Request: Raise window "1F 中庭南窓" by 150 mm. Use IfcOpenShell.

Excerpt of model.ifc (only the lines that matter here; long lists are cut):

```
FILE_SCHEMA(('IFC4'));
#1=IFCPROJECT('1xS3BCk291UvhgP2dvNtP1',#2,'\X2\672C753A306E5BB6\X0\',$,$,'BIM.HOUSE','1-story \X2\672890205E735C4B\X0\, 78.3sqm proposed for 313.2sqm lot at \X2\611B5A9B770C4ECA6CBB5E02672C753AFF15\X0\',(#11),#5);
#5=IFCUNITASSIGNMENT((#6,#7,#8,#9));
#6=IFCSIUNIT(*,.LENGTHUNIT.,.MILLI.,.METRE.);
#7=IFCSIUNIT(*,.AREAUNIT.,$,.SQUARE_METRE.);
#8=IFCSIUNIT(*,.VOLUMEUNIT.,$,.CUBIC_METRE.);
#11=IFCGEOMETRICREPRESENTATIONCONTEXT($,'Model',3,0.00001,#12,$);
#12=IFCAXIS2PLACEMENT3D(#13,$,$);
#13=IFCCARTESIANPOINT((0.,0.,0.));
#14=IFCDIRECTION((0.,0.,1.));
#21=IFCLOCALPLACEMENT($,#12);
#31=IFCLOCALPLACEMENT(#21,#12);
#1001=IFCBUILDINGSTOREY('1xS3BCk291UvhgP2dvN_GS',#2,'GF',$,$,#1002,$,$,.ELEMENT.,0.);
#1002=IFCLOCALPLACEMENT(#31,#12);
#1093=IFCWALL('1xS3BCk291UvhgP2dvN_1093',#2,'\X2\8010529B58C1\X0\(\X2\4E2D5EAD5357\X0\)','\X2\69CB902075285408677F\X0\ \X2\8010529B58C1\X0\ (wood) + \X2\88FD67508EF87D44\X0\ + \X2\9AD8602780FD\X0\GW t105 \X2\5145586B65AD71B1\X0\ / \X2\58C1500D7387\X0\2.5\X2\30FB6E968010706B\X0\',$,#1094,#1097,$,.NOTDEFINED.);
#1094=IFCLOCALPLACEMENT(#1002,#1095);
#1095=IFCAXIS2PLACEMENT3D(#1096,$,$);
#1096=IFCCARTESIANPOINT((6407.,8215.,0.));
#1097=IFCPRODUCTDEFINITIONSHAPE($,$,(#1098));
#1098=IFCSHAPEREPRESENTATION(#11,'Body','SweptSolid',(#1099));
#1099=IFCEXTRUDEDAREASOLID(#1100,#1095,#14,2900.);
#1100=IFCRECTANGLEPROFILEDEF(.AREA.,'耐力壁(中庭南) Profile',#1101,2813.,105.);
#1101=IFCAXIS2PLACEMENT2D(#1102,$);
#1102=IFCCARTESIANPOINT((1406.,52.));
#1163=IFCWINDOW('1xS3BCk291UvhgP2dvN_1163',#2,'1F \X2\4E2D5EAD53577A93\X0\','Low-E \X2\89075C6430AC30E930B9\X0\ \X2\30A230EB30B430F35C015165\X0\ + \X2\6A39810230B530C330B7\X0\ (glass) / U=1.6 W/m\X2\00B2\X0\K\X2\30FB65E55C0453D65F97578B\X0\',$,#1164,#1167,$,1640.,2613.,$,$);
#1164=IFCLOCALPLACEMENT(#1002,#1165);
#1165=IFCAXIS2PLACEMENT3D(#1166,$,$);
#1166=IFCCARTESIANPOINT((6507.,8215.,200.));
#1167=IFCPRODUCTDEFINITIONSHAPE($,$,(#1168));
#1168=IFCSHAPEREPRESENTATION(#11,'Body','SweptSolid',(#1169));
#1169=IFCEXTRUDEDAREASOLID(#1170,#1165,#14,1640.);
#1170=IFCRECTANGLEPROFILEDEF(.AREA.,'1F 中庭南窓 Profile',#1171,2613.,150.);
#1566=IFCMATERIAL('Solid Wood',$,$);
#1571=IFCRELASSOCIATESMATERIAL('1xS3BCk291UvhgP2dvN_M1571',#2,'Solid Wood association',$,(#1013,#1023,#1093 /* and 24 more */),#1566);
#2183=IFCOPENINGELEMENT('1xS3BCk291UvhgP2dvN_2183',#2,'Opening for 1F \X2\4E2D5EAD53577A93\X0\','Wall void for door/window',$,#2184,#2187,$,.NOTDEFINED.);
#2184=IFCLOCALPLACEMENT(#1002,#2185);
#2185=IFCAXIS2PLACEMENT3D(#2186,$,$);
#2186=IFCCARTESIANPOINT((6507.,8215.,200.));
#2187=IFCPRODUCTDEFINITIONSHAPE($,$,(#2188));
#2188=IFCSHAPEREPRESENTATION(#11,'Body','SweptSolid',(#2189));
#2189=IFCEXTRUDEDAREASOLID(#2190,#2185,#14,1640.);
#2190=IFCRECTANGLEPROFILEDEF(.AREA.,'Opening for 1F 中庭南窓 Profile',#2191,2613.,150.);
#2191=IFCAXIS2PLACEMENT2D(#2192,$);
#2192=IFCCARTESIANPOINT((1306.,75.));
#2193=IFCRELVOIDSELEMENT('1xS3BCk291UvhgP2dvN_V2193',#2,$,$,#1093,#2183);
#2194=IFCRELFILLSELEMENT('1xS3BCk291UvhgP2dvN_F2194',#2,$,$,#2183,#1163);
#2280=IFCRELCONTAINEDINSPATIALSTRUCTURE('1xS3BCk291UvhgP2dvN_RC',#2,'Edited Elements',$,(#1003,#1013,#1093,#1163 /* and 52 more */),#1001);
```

```python
import numpy as np
import ifcopenshell
import ifcopenshell.api.geometry
import ifcopenshell.util.placement
import ifcopenshell.util.unit

model = ifcopenshell.open("model.ifc")
unit_scale = ifcopenshell.util.unit.calculate_unit_scale(model)

window = model.by_guid("1xS3BCk291UvhgP2dvN_1163")
opening = window.FillsVoids[0].RelatingOpeningElement
dz = 0.15 / unit_scale

shift = np.array([0.0, 0.0, dz])
# The window is not placed relative to its opening, so move both.
for product in (opening, window):
    matrix = ifcopenshell.util.placement.get_local_placement(product.ObjectPlacement)
    matrix[:3, 3] += shift
    ifcopenshell.api.geometry.edit_object_placement(model, product=product, matrix=matrix, is_si=False)

print(f"moved by {dz * unit_scale:+.3f} m")

model.write("model_edited.ifc")
```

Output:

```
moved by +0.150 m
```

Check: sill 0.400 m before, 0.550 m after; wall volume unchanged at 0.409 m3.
